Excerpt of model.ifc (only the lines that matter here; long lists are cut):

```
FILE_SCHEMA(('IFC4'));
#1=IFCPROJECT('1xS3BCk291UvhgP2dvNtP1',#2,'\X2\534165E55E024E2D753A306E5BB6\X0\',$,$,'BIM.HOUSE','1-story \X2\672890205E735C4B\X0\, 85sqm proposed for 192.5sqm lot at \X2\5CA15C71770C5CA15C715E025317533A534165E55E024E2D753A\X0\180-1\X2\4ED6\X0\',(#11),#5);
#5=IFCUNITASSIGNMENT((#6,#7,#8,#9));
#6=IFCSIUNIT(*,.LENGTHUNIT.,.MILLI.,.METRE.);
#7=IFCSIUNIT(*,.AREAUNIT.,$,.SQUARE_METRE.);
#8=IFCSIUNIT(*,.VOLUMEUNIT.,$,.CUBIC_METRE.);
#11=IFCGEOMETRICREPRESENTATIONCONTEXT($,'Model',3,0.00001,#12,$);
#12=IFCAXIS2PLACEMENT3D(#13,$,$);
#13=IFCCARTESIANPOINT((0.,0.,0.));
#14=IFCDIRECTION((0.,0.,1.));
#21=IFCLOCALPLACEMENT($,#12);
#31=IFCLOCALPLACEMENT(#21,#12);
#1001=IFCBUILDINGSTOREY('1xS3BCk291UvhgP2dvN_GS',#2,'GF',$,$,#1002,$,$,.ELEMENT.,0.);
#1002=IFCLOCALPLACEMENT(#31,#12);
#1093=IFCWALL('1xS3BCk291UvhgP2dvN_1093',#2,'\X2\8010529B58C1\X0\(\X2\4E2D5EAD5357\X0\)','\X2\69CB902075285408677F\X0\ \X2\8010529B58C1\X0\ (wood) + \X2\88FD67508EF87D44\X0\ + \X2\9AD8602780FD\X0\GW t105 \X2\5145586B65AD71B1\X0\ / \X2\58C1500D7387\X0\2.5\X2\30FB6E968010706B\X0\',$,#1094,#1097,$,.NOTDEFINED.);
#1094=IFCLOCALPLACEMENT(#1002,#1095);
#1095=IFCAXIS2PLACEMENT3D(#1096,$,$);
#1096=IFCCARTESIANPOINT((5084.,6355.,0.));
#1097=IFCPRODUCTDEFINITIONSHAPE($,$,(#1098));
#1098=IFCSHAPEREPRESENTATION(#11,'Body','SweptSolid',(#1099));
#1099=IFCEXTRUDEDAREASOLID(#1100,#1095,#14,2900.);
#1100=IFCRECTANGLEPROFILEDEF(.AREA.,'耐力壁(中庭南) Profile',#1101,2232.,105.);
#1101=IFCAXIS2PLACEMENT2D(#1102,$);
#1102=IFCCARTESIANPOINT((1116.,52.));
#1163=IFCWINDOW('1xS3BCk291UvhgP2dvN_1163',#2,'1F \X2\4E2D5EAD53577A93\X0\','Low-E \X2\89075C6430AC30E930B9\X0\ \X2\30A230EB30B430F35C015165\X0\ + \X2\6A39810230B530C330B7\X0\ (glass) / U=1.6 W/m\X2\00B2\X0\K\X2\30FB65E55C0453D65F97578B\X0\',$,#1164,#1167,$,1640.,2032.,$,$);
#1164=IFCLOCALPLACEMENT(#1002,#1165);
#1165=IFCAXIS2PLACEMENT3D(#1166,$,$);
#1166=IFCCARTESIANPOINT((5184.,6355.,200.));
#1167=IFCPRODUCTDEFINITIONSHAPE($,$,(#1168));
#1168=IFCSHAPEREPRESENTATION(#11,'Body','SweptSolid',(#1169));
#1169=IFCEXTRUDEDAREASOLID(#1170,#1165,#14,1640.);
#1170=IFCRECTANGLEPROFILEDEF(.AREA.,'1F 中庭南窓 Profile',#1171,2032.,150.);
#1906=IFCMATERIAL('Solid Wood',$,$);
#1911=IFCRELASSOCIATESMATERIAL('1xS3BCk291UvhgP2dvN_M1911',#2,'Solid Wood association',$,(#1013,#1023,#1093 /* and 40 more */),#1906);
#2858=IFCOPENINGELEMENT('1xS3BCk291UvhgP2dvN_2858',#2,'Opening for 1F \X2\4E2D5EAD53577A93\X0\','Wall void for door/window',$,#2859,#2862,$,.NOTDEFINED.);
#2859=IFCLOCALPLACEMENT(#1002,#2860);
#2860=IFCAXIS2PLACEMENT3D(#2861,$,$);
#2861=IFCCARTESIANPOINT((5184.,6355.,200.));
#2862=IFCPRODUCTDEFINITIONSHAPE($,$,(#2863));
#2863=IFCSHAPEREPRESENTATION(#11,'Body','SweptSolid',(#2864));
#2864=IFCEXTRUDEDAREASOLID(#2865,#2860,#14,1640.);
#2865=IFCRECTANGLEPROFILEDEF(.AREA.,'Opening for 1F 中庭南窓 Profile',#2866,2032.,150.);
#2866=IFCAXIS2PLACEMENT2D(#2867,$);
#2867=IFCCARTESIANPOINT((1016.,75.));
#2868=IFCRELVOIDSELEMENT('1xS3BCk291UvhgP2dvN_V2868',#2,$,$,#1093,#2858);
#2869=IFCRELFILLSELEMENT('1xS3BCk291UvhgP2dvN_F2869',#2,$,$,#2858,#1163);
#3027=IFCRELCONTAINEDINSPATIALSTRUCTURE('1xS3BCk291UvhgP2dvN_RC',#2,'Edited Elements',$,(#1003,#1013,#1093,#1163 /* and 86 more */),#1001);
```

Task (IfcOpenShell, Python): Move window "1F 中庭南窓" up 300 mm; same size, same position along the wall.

```python
import numpy as np
import ifcopenshell
import ifcopenshell.api.geometry
import ifcopenshell.util.placement
import ifcopenshell.util.unit

model = ifcopenshell.open("model.ifc")
unit_scale = ifcopenshell.util.unit.calculate_unit_scale(model)

window = model.by_id(1163)
opening = window.FillsVoids[0].RelatingOpeningElement
dz = 0.3 / unit_scale

shift = np.array([0.0, 0.0, dz])
# The window is not placed relative to its opening, so move both.
for product in (opening, window):
    matrix = ifcopenshell.util.placement.get_local_placement(product.ObjectPlacement)
    matrix[:3, 3] += shift
    ifcopenshell.api.geometry.edit_object_placement(model, product=product, matrix=matrix, is_si=False)

print(f"moved by {dz * unit_scale:+.3f} m")

model.write("model_updated.ifc")
```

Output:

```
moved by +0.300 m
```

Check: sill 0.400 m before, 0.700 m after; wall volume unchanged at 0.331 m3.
